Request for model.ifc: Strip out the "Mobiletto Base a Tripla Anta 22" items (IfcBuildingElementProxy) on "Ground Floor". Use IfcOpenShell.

First a look at what the model holds.

```python
import ifcopenshell
import ifcopenshell.util.element

model = ifcopenshell.open("model.ifc")
print(model.schema)
storey = next(s for s in model.by_type("IfcBuildingStorey") if s.Name == "Ground Floor")
proxies = [e for e in ifcopenshell.util.element.get_decomposition(storey) if e.is_a("IfcBuildingElementProxy")]
seen = {}
for e in proxies:
    element_type = ifcopenshell.util.element.get_type(e)
    name = element_type.Name if element_type not in (None, e) else None
    seen[name] = seen.get(name, 0) + 1
for name, count in sorted(seen.items(), key=str):
    print(count, "x", name)
```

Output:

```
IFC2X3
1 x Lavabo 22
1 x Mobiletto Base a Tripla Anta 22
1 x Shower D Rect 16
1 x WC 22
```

```python
import ifcopenshell
import ifcopenshell.api.root
import ifcopenshell.util.element

model = ifcopenshell.open("model.ifc")

storey = next(s for s in model.by_type("IfcBuildingStorey") if s.Name == "Ground Floor")
proxies = [e for e in ifcopenshell.util.element.get_decomposition(storey) if e.is_a("IfcBuildingElementProxy")]
targets = [e for e in proxies if (t := ifcopenshell.util.element.get_type(e)) not in (None, e) and t.Name == "Mobiletto Base a Tripla Anta 22"]

for e in targets:
    ifcopenshell.api.root.remove_product(model, product=e)
print(len(targets), "removed")

model.write("model-out.ifc")
```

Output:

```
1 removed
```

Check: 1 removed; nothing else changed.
